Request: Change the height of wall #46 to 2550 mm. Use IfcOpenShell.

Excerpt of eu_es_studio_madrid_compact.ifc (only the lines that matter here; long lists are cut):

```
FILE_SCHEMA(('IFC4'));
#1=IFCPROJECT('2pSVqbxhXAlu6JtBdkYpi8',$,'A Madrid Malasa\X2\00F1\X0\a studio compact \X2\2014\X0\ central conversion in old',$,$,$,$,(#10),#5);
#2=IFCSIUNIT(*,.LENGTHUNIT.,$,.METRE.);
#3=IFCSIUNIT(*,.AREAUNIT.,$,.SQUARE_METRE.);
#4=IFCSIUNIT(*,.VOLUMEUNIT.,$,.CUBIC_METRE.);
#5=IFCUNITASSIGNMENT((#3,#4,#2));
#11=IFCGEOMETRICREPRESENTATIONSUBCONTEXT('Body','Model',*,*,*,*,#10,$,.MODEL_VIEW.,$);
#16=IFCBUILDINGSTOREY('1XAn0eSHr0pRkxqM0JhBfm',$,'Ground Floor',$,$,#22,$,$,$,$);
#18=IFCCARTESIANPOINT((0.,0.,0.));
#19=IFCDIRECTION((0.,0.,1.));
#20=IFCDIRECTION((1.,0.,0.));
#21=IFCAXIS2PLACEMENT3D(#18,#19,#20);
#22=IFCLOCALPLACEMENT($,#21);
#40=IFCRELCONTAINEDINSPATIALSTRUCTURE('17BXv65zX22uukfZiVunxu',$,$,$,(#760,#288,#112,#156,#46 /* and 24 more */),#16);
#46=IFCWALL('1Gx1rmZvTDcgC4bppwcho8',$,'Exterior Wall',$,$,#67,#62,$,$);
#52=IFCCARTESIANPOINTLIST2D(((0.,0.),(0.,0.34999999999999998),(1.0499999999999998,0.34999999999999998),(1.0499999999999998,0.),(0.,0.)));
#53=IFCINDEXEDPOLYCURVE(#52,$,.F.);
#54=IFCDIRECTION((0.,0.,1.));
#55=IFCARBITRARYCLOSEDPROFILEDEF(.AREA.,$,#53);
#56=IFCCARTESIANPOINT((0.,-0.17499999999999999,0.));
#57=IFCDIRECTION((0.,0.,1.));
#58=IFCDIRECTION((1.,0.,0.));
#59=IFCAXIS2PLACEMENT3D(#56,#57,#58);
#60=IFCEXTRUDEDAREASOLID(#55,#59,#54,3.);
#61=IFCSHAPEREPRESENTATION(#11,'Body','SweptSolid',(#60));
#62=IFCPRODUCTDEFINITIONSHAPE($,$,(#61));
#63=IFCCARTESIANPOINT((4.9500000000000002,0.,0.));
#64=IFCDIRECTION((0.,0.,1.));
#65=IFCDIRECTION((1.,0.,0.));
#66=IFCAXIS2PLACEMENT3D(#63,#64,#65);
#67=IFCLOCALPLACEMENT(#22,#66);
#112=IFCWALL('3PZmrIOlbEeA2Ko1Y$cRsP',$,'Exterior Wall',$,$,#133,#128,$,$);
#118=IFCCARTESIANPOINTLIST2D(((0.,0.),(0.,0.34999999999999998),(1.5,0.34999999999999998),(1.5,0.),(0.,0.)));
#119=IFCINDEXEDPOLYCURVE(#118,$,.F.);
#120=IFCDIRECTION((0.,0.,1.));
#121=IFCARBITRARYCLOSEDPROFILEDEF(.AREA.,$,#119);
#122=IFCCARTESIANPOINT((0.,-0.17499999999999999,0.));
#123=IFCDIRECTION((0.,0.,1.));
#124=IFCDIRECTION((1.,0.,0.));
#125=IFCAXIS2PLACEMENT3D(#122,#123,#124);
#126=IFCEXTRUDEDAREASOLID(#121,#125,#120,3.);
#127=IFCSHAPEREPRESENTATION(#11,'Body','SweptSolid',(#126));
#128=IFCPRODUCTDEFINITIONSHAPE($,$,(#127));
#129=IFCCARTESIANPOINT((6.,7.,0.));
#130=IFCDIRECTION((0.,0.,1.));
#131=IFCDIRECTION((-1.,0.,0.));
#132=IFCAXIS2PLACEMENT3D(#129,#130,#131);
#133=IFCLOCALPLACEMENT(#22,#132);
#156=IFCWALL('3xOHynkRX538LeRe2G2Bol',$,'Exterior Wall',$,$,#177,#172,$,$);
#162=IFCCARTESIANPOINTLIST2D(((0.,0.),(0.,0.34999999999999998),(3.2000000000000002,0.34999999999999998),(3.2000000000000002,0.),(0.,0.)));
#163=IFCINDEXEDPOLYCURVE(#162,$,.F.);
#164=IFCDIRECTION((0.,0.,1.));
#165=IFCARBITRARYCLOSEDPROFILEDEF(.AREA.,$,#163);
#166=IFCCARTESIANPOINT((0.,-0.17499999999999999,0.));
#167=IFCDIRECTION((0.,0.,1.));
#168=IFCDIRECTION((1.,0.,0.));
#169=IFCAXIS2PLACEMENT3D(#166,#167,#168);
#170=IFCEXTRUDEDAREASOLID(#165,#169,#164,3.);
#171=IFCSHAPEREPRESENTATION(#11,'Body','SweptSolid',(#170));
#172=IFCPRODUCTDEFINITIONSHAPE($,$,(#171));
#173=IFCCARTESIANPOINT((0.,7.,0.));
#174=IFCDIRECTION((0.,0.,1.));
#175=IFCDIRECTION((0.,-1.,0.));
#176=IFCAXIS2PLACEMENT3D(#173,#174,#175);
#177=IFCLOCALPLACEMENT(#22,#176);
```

```python
import ifcopenshell
import ifcopenshell.geom
import ifcopenshell.util.representation
import ifcopenshell.util.shape
import ifcopenshell.util.unit

model = ifcopenshell.open("eu_es_studio_madrid_compact.ifc")
unit_scale = ifcopenshell.util.unit.calculate_unit_scale(model)
settings = ifcopenshell.geom.settings()


def volume(element):
    """Net volume in cubic metres, openings subtracted."""
    shape = ifcopenshell.geom.create_shape(settings, element)
    return ifcopenshell.util.shape.get_volume(shape.geometry)


wall = model.by_guid("1Gx1rmZvTDcgC4bppwcho8")
before = volume(wall)

body = ifcopenshell.util.representation.get_representation(wall, "Model", "Body")
solid = body.Items[0]
old_height = solid.Depth
solid.Depth = 2.55 / unit_scale
after = volume(wall)

print(f"height {old_height:g} -> {solid.Depth:g}, volume {before:.3f} -> {after:.3f} m3")

model.write("eu_es_studio_madrid_compact-out.ifc")
```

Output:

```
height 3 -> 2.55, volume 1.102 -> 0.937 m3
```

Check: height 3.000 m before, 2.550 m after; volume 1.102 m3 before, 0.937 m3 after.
